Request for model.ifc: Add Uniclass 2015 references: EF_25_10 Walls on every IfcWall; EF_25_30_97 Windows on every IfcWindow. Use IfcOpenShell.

First a look at what the model holds.

```python
import ifcopenshell

model = ifcopenshell.open("model.ifc")
print(model.schema)
print("classifications:", [c.Name for c in model.by_type("IfcClassification")])
for ifc_class in ("IfcDoor", "IfcRoof", "IfcStair", "IfcWall", "IfcWindow"):
    print(ifc_class, len(model.by_type(ifc_class)))
```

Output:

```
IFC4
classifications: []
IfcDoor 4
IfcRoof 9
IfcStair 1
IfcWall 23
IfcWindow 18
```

```python
import ifcopenshell
import ifcopenshell.api.classification

model = ifcopenshell.open("model.ifc")

system = ifcopenshell.api.classification.add_classification(model, classification="Uniclass 2015")

codes = {
    "IfcWall": ("EF_25_10", "Walls"),
    "IfcWindow": ("EF_25_30_97", "Windows"),
}
for ifc_class, (code, name) in codes.items():
    products = model.by_type(ifc_class)
    ifcopenshell.api.classification.add_reference(
        model, products=products, classification=system, identification=code, name=name
    )
    print(code, len(products))

model.write("model_updated.ifc")
```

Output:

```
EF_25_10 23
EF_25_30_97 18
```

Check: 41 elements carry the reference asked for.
